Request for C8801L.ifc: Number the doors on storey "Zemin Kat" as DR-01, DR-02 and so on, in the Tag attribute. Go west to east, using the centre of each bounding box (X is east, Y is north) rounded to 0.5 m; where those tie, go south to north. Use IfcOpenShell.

First a look at what the model holds.

```python
import ifcopenshell
import ifcopenshell.util.element
import ifcopenshell.util.placement

model = ifcopenshell.open("C8801L.ifc")
print(model.schema)
storey = next(s for s in model.by_type("IfcBuildingStorey") if s.Name == "Zemin Kat")
doors = [e for e in ifcopenshell.util.element.get_decomposition(storey) if e.is_a("IfcDoor")]
for e in sorted(doors, key=lambda e: e.id()):
    origin = ifcopenshell.util.placement.get_local_placement(e.ObjectPlacement)[:3, 3]
    print(e.id(), e.Tag, e.Name, origin.round(2) + 0.0, sep=" | ")
```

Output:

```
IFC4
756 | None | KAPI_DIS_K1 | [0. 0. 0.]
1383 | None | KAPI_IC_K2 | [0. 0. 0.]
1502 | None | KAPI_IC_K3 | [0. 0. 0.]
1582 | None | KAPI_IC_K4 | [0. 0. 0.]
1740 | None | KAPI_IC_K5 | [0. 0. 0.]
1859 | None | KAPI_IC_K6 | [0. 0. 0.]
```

```python
import ifcopenshell
import ifcopenshell.geom
import ifcopenshell.util.element
import ifcopenshell.util.shape

model = ifcopenshell.open("C8801L.ifc")
settings = ifcopenshell.geom.settings()
settings.set("use-world-coords", True)


def centre(element):
    shape = ifcopenshell.geom.create_shape(settings, element)
    return ifcopenshell.util.shape.get_bbox_centroid(shape.geometry)


storey = next(s for s in model.by_type("IfcBuildingStorey") if s.Name == "Zemin Kat")
doors = [e for e in ifcopenshell.util.element.get_decomposition(storey) if e.is_a("IfcDoor")]

# Insertion points can sit at a corner or the storey origin, so sort by the geometry (in metres).
centres = {e: centre(e) for e in doors}
doors.sort(key=lambda e: (round(centres[e][0] / 0.5), centres[e][1]))

for i, e in enumerate(doors, start=1):
    number = f"DR-{i:02d}"
    e.Tag = number
    print(e.id(), number)

model.write("C8801L_rev.ifc")
```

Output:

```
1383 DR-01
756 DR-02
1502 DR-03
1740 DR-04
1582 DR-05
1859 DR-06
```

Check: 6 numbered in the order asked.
